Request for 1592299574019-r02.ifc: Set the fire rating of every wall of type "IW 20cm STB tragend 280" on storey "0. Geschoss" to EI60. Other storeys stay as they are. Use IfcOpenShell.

First a look at what the model holds.

```python
import ifcopenshell
import ifcopenshell.util.element

model = ifcopenshell.open("1592299574019-r02.ifc")
print(model.schema)
storey = next(s for s in model.by_type("IfcBuildingStorey") if s.Name == "0. Geschoss")
walls = [e for e in ifcopenshell.util.element.get_decomposition(storey) if e.is_a("IfcWall")]
seen = {}
for e in walls:
    element_type = ifcopenshell.util.element.get_type(e)
    key = (element_type.Name if element_type != e and element_type else None, ifcopenshell.util.element.get_pset(e, "Pset_WallCommon", "FireRating"))
    seen[key] = seen.get(key, 0) + 1
for (name, value), count in sorted(seen.items(), key=str):
    print(count, "x", name, "|", value)
```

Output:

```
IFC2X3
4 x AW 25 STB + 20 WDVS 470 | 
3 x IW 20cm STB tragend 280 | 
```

```python
import ifcopenshell
import ifcopenshell.api.pset
import ifcopenshell.util.element

model = ifcopenshell.open("1592299574019-r02.ifc")

storey = next(s for s in model.by_type("IfcBuildingStorey") if s.Name == "0. Geschoss")
walls = [e for e in ifcopenshell.util.element.get_decomposition(storey) if e.is_a("IfcWall")]

count = 0
for e in walls:
    element_type = ifcopenshell.util.element.get_type(e)
    if element_type in (None, e) or element_type.Name != "IW 20cm STB tragend 280":
        continue
    # add_pset returns the element's existing set when there is one.
    pset = ifcopenshell.api.pset.add_pset(model, product=e, name="Pset_WallCommon")
    ifcopenshell.api.pset.edit_pset(model, pset=pset, properties={"FireRating": "EI60"})
    count += 1

print(count, "walls updated")

model.write("1592299574019-r02_updated.ifc")
```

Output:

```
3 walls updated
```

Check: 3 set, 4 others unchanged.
